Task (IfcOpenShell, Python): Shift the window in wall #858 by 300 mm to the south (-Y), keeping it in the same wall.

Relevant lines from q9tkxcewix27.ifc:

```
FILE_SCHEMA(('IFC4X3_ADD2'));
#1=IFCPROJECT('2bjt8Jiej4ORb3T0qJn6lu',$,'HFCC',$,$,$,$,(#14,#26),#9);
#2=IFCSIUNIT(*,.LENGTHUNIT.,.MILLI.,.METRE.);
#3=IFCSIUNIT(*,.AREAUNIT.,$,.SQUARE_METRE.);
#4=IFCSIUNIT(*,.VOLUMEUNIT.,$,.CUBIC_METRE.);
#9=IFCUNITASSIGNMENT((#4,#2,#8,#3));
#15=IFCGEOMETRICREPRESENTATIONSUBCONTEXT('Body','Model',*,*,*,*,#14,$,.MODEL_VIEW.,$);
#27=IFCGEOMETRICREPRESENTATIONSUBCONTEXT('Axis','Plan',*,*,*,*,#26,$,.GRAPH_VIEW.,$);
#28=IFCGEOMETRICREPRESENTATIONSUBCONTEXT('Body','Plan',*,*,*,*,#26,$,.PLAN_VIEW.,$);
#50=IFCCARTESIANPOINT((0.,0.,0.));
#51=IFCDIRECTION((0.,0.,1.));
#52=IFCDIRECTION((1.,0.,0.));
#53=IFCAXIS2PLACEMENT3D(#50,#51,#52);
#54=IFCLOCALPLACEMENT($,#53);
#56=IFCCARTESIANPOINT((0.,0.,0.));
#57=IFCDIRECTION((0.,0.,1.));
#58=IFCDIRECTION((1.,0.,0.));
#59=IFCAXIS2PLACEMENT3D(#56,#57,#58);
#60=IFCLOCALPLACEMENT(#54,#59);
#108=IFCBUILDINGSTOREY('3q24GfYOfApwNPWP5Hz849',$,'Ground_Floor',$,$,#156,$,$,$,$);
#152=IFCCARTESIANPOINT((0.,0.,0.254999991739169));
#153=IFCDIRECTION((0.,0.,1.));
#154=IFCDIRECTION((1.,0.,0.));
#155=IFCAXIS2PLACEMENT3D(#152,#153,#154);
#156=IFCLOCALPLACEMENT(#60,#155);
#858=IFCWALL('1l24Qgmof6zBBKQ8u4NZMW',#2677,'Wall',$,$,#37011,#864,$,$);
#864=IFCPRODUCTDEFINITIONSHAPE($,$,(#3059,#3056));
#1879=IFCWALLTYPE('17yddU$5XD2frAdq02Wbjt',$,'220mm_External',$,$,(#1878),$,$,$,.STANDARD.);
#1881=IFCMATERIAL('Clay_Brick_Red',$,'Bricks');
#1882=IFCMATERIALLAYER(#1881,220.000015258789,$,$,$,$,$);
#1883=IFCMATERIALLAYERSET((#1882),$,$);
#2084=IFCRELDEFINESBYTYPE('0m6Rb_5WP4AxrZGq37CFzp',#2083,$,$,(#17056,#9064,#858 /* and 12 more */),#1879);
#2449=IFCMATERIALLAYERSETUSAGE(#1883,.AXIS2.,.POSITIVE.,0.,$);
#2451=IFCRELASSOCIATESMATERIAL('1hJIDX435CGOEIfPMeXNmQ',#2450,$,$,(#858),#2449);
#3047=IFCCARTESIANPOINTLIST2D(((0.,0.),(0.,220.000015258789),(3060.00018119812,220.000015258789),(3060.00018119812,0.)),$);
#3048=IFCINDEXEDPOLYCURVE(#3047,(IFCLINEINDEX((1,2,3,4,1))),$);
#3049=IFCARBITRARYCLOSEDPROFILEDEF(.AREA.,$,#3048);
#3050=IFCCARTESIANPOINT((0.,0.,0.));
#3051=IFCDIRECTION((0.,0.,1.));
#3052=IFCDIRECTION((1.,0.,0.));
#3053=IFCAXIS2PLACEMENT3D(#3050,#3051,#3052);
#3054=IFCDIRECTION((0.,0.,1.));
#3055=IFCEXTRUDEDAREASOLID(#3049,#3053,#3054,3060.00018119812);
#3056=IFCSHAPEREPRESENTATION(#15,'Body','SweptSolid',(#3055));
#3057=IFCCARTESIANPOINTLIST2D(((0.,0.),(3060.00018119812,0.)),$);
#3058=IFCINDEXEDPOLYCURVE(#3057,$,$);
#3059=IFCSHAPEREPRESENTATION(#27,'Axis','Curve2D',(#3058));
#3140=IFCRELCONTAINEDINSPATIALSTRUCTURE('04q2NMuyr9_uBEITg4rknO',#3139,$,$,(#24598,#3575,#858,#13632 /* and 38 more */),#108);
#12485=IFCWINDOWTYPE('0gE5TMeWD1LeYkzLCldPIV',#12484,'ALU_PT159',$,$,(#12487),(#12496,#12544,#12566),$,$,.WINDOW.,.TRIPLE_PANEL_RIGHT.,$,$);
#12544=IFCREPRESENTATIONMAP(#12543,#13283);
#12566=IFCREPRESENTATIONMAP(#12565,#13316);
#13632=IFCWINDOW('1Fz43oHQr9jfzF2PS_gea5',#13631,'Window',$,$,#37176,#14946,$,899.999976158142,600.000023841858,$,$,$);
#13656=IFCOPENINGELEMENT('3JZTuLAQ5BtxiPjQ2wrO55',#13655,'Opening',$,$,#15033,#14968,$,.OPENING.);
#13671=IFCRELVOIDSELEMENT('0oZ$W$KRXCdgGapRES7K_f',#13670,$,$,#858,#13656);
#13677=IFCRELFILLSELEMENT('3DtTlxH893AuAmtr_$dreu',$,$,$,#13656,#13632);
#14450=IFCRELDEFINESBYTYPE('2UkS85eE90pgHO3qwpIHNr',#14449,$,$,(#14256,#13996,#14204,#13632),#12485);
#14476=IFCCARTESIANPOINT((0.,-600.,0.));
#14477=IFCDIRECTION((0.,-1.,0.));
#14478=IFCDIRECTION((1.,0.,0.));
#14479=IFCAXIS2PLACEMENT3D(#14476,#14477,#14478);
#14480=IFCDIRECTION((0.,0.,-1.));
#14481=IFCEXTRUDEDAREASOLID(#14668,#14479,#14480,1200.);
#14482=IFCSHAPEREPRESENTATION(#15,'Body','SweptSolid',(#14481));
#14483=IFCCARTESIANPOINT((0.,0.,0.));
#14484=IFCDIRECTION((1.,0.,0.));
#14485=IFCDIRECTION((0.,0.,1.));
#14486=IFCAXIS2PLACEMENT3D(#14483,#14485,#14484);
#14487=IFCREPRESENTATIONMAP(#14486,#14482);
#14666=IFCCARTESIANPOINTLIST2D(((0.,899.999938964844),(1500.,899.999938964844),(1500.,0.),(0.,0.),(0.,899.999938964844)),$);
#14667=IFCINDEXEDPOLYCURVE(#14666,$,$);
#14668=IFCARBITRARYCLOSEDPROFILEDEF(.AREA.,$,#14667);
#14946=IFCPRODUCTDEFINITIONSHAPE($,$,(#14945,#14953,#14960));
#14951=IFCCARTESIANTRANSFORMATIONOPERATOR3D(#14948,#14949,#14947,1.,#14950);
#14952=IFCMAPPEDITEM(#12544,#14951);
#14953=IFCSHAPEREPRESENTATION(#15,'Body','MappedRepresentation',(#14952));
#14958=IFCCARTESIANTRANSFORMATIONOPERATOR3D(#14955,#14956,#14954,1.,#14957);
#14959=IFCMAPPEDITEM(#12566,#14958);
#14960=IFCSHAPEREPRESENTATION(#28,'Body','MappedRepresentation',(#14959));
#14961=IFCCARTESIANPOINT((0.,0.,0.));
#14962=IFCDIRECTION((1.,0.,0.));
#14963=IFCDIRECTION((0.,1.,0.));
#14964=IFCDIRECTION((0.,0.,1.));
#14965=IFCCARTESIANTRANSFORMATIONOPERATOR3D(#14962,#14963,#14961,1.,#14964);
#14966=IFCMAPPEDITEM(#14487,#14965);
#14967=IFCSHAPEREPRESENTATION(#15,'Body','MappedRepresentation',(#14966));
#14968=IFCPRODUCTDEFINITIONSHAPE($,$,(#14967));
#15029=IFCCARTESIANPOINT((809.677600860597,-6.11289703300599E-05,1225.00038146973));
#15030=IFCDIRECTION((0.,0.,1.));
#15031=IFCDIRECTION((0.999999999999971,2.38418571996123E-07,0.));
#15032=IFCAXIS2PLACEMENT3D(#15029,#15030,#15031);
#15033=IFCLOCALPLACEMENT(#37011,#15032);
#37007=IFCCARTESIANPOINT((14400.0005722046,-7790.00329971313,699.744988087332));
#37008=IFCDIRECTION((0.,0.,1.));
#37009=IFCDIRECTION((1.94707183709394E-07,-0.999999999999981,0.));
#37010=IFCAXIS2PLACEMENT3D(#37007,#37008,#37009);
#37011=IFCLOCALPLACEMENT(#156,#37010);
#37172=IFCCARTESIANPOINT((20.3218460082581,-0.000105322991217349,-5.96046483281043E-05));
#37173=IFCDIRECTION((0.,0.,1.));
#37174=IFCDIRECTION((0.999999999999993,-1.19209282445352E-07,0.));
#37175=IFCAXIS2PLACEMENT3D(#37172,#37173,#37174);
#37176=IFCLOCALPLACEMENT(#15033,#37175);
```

```python
import ifcopenshell
import ifcopenshell.api.geometry
import ifcopenshell.util.placement
import ifcopenshell.util.unit

model = ifcopenshell.open("q9tkxcewix27.ifc")
unit_scale = ifcopenshell.util.unit.calculate_unit_scale(model)

window = model.by_id(13632)
opening = window.FillsVoids[0].RelatingOpeningElement
wall = opening.VoidsElements[0].RelatingBuildingElement

wall_matrix = ifcopenshell.util.placement.get_local_placement(wall.ObjectPlacement)
shift = wall_matrix[:3, 0] * 0.3 / unit_scale
before = ifcopenshell.util.placement.get_local_placement(window.ObjectPlacement)[:3, 3].copy()

# The window is placed relative to its opening, so it follows when the opening moves.
matrix = ifcopenshell.util.placement.get_local_placement(opening.ObjectPlacement)
matrix[:3, 3] += shift
ifcopenshell.api.geometry.edit_object_placement(
    model, product=opening, matrix=matrix, is_si=False, should_transform_children=True
)

after = ifcopenshell.util.placement.get_local_placement(window.ObjectPlacement)[:3, 3]
print("window moved by", (after - before).round(3) + 0.0)

model.write("q9tkxcewix27_edited.ifc")
```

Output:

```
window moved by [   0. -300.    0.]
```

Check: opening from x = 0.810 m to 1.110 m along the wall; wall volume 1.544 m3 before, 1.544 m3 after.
